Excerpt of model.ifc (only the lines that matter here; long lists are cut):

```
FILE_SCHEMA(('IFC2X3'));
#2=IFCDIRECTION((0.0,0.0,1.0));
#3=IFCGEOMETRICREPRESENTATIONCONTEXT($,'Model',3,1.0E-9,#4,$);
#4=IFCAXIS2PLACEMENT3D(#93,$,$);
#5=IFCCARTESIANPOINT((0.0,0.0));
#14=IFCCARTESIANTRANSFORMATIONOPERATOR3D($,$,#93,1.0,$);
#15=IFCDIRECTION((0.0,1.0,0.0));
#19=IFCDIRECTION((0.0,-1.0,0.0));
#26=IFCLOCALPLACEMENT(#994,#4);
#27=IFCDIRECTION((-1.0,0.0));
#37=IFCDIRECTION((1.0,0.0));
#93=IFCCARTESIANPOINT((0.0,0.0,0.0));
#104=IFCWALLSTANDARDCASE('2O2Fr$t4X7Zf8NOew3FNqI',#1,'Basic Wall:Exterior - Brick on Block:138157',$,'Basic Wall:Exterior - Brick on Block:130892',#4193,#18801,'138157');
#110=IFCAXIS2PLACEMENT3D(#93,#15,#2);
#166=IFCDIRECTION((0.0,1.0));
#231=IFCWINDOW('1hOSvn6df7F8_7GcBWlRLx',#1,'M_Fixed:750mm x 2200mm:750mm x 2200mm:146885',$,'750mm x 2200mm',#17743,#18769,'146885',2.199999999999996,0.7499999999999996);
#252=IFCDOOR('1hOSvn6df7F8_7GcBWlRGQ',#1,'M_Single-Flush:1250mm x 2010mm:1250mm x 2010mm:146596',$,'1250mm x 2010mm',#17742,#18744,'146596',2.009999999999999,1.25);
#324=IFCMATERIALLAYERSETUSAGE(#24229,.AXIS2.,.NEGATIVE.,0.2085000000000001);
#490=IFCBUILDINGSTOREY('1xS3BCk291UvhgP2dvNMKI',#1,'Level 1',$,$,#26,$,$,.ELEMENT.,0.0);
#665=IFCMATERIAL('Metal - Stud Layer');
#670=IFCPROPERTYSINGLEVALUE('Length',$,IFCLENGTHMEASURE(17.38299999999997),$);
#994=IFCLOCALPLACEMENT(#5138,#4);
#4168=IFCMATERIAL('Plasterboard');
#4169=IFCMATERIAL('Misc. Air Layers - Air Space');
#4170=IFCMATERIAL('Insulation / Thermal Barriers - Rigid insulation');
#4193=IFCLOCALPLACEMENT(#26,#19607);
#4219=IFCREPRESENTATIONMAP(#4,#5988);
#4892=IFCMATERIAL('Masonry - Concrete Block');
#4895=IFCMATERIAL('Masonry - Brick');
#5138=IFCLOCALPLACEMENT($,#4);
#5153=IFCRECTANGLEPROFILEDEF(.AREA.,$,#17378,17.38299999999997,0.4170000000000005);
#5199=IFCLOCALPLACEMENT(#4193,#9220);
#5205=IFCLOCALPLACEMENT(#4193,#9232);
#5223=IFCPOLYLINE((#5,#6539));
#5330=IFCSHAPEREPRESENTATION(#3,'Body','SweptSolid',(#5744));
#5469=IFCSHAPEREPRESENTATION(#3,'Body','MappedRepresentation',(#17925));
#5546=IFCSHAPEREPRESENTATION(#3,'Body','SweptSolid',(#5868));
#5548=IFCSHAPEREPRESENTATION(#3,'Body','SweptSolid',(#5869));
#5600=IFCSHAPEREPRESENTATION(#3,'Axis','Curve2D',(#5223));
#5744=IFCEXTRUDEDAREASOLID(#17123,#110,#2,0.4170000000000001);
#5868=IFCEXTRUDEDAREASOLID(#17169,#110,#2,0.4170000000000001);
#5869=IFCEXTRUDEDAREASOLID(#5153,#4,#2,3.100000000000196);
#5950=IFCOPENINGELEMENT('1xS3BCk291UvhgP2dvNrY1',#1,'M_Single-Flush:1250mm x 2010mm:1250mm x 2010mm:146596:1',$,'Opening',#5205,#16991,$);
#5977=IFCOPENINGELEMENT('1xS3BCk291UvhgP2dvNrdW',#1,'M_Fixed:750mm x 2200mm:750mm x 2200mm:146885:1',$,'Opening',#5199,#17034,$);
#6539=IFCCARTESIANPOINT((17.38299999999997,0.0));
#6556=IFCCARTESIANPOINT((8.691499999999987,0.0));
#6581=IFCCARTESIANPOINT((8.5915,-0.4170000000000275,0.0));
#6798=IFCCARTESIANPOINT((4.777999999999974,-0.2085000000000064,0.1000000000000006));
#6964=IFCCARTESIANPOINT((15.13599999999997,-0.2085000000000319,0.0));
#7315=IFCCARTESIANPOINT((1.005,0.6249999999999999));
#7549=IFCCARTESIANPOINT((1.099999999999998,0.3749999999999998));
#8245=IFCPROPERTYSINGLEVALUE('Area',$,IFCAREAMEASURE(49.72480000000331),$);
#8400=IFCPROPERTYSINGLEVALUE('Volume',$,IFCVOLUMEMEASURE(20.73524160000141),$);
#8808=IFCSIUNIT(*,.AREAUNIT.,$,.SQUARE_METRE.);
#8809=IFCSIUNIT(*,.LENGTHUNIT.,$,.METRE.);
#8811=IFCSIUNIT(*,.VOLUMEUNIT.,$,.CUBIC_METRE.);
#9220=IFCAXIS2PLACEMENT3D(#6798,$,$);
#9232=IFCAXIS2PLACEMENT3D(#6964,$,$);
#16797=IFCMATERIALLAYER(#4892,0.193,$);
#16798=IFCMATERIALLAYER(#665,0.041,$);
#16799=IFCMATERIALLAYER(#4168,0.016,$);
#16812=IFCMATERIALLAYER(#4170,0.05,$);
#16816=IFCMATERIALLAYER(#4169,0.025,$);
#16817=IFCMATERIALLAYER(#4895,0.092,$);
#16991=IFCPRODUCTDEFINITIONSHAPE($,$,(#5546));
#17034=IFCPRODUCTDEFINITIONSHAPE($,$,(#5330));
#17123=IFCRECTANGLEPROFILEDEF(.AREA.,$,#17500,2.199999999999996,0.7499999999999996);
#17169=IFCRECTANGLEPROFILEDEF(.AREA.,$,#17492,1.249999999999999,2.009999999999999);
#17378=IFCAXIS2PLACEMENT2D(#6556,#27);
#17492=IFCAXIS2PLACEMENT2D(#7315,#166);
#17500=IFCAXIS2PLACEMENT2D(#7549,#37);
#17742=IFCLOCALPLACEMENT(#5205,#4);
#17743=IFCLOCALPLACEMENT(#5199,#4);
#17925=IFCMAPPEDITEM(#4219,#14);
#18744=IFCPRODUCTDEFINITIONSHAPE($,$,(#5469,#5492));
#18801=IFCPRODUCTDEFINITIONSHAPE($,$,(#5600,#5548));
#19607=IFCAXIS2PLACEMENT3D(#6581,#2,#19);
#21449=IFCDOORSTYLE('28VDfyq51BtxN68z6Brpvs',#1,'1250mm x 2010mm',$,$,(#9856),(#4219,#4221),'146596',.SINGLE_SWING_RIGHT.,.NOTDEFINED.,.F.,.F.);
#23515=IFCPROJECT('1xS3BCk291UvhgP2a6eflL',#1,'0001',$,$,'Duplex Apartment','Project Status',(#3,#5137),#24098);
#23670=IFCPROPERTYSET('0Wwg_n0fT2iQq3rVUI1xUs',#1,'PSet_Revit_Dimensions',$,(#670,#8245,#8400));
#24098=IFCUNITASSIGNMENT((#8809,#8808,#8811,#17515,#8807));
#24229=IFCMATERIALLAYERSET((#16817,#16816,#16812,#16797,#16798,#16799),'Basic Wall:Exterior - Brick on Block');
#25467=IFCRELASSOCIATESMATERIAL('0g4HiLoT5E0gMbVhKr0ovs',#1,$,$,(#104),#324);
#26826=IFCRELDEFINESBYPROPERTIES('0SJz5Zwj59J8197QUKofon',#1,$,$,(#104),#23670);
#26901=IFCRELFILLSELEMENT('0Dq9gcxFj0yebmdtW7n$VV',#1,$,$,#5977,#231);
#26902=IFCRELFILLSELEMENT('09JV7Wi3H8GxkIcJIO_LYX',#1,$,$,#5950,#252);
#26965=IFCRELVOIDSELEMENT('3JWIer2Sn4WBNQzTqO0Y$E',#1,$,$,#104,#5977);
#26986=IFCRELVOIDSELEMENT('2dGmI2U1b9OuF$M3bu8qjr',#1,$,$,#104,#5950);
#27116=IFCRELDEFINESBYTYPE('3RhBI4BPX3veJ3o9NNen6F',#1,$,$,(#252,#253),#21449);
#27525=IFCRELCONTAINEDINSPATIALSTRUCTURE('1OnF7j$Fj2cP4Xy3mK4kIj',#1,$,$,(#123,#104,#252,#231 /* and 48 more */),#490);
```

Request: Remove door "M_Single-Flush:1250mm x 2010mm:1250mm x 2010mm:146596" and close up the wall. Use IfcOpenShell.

```python
import ifcopenshell
import ifcopenshell.api.feature
import ifcopenshell.api.pset
import ifcopenshell.api.root
import ifcopenshell.geom
import ifcopenshell.util.element
import ifcopenshell.util.shape
import ifcopenshell.util.unit

model = ifcopenshell.open("model.ifc")
area_scale = ifcopenshell.util.unit.calculate_unit_scale(model, "AREAUNIT")
volume_scale = ifcopenshell.util.unit.calculate_unit_scale(model, "VOLUMEUNIT")
settings = ifcopenshell.geom.settings()


def volume(element):
    """Net volume in cubic metres, openings subtracted."""
    shape = ifcopenshell.geom.create_shape(settings, element)
    return ifcopenshell.util.shape.get_volume(shape.geometry)


door = model.by_id(252)
opening = door.FillsVoids[0].RelatingOpeningElement
wall = opening.VoidsElements[0].RelatingBuildingElement
before = volume(wall)

ifcopenshell.api.root.remove_product(model, product=door)
ifcopenshell.api.feature.remove_feature(model, feature=opening)

after = volume(wall)
thickness = 0.417  # wall thickness in metres

# Update the wall's stored quantities.
pset = model.by_id(ifcopenshell.util.element.get_pset(wall, "PSet_Revit_Dimensions", should_inherit=False)["id"])
ifcopenshell.api.pset.edit_pset(model, pset=pset, properties={
    "Area": model.create_entity("IfcAreaMeasure", after / thickness / area_scale),
    "Volume": model.create_entity("IfcVolumeMeasure", after / volume_scale),
})

print(f"wall volume {before:.3f} -> {after:.3f} m3")

model.write("model_v2.ifc")
```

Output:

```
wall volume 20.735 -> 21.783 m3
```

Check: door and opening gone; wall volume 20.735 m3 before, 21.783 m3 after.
